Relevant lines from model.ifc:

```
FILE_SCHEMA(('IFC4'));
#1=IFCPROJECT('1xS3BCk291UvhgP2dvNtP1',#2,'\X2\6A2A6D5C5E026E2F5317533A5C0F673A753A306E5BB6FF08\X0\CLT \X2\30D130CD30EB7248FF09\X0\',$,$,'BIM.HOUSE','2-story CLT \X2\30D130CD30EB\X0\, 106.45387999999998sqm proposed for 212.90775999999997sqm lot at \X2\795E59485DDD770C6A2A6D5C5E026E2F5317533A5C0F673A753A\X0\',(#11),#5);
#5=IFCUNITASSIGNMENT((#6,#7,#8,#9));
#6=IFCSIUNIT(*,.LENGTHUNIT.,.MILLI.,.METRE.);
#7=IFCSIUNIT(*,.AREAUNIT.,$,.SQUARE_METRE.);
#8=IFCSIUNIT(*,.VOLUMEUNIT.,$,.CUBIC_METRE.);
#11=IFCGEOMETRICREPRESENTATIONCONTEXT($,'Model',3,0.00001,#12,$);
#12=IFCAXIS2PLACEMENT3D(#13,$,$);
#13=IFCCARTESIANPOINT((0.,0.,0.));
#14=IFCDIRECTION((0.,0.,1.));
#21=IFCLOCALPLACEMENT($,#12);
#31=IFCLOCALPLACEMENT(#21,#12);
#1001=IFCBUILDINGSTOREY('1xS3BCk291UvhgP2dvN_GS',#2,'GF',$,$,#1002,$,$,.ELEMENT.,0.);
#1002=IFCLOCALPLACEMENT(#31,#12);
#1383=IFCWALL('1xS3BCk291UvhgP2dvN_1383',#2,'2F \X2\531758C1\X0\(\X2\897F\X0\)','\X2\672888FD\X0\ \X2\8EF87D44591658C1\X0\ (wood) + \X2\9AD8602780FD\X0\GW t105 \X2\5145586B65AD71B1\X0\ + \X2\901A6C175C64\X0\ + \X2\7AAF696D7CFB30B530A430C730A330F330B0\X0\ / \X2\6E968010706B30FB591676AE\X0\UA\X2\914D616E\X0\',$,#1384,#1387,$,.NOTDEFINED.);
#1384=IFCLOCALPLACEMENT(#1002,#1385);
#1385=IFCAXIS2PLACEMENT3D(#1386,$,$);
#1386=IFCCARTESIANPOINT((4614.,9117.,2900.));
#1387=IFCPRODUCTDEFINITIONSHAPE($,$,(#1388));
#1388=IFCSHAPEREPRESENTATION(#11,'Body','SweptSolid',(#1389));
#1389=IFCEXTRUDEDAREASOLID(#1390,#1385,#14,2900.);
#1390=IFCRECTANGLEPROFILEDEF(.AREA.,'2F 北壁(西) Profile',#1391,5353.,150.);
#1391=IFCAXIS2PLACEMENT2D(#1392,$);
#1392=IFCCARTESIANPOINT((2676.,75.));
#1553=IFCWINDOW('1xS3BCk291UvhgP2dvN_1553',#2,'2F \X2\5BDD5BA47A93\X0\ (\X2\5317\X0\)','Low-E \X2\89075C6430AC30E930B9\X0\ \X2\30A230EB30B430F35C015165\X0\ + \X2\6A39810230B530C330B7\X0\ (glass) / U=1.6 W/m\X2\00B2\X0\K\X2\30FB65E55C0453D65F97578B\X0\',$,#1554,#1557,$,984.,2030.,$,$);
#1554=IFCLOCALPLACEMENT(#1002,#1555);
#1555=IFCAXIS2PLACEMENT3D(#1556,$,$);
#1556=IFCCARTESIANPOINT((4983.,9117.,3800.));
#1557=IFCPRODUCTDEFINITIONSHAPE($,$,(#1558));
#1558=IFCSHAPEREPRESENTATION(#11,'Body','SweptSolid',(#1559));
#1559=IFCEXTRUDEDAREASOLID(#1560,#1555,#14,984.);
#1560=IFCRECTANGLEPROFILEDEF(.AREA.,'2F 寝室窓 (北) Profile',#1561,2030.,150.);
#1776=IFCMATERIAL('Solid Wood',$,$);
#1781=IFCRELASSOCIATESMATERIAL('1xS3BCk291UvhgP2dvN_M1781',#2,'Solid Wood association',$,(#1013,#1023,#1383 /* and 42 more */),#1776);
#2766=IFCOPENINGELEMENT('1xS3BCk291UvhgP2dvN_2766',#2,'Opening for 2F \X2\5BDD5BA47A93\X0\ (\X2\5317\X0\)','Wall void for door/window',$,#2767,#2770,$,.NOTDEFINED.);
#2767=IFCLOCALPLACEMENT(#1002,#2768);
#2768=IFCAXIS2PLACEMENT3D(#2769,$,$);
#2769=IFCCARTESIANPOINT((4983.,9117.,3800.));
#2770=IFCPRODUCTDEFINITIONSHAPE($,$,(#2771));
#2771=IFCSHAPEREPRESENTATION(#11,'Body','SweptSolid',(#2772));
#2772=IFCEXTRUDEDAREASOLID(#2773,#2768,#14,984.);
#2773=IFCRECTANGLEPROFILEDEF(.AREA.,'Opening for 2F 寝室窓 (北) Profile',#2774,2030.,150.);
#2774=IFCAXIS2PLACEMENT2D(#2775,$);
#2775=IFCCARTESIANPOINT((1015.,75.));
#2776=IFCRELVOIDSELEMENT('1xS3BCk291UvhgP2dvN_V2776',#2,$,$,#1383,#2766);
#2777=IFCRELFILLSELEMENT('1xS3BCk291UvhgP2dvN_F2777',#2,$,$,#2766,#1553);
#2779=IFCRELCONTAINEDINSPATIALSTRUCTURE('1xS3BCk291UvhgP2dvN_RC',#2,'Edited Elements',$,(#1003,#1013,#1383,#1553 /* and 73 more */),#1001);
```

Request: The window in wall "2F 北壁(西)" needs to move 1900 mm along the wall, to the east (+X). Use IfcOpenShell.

```python
import ifcopenshell
import ifcopenshell.api.geometry
import ifcopenshell.util.placement
import ifcopenshell.util.unit

model = ifcopenshell.open("model.ifc")
unit_scale = ifcopenshell.util.unit.calculate_unit_scale(model)

window = model.by_guid("1xS3BCk291UvhgP2dvN_1553")
opening = window.FillsVoids[0].RelatingOpeningElement
wall = opening.VoidsElements[0].RelatingBuildingElement

wall_matrix = ifcopenshell.util.placement.get_local_placement(wall.ObjectPlacement)
shift = wall_matrix[:3, 0] * 1.9 / unit_scale
before = ifcopenshell.util.placement.get_local_placement(window.ObjectPlacement)[:3, 3].copy()

# The window is not placed relative to its opening, so move both.
for product in (opening, window):
    matrix = ifcopenshell.util.placement.get_local_placement(product.ObjectPlacement)
    matrix[:3, 3] += shift
    ifcopenshell.api.geometry.edit_object_placement(model, product=product, matrix=matrix, is_si=False)

after = ifcopenshell.util.placement.get_local_placement(window.ObjectPlacement)[:3, 3]
print("window moved by", (after - before).round(3) + 0.0)

model.write("model_v2.ifc")
```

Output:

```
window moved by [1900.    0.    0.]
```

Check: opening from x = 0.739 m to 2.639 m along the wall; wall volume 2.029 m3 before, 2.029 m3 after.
